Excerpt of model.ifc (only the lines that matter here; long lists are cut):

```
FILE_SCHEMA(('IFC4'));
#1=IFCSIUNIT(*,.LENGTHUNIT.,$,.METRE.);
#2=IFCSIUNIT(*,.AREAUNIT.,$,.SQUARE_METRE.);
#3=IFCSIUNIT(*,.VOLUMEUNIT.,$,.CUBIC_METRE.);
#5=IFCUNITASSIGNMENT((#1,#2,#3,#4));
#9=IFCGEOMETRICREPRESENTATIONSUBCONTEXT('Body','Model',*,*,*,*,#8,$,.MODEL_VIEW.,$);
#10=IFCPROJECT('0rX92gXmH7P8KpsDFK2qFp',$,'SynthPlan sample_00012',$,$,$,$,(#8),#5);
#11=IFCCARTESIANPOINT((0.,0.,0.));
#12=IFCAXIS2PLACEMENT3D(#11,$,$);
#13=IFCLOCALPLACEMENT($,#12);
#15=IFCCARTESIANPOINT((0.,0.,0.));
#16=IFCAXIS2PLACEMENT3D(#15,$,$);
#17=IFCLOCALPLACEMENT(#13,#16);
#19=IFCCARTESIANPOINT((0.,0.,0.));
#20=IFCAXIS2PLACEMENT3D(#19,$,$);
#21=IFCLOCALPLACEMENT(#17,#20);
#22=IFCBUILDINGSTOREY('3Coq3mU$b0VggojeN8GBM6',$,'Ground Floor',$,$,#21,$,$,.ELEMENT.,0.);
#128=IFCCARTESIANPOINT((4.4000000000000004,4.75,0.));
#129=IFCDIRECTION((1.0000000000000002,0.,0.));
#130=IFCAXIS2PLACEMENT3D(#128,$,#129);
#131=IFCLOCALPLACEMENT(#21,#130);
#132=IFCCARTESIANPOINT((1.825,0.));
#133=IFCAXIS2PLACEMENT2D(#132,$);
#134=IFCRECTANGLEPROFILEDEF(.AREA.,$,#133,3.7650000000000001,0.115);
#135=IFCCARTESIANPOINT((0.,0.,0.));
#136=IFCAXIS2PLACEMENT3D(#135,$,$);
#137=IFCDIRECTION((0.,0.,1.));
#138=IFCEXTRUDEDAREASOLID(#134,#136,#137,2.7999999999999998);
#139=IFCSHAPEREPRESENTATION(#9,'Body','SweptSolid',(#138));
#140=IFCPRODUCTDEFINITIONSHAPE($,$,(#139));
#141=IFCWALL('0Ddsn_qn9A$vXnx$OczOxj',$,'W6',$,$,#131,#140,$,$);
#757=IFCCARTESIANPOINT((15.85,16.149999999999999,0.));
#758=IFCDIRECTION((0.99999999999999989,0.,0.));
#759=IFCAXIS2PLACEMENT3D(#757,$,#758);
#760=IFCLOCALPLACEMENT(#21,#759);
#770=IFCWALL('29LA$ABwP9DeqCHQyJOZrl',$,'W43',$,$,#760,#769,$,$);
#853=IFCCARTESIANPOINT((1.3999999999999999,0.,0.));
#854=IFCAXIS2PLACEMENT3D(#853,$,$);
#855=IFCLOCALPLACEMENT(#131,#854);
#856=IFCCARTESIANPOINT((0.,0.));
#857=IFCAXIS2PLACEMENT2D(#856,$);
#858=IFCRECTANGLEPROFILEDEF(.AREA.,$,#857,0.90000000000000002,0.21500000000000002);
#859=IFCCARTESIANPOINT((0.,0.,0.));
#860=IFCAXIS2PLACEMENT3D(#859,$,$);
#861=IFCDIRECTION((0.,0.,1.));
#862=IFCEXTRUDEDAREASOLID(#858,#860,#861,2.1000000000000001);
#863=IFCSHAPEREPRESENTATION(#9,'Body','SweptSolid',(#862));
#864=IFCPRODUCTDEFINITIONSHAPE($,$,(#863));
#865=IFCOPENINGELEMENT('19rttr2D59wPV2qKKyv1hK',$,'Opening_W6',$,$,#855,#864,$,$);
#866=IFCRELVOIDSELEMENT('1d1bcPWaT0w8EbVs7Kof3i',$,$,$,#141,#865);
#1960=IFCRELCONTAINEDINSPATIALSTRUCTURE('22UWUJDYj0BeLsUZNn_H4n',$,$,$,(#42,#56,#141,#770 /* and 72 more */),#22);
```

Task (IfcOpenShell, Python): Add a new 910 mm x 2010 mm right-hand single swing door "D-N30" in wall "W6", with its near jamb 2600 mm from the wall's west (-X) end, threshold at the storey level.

```python
import numpy as np
import ifcopenshell
import ifcopenshell.api.feature
import ifcopenshell.api.geometry
import ifcopenshell.api.root
import ifcopenshell.api.spatial
import ifcopenshell.geom
import ifcopenshell.util.element
import ifcopenshell.util.placement
import ifcopenshell.util.representation
import ifcopenshell.util.shape
import ifcopenshell.util.unit

model = ifcopenshell.open("model.ifc")
unit_scale = ifcopenshell.util.unit.calculate_unit_scale(model)
settings = ifcopenshell.geom.settings()


def volume(element):
    """Net volume in cubic metres, openings subtracted."""
    shape = ifcopenshell.geom.create_shape(settings, element)
    return ifcopenshell.util.shape.get_volume(shape.geometry)


wall = model.by_guid("0Ddsn_qn9A$vXnx$OczOxj")
storey = ifcopenshell.util.element.get_container(wall, ifc_class="IfcBuildingStorey")
context = ifcopenshell.util.representation.get_context(model, "Model", "Body", "MODEL_VIEW")
before = volume(wall)

width, height, from_end, sill = 0.91, 2.01, 2.6, 0.0  # metres

# The wall runs along its own X axis, and the end named is its -X end.
wall_shape = ifcopenshell.geom.create_shape(settings, wall)
x, y, z = ifcopenshell.util.shape.get_vertices(wall_shape.geometry).T
start = x.min() + from_end
face, thickness = float(y.min()), float(y.max() - y.min())
wall_matrix = ifcopenshell.util.placement.get_local_placement(wall.ObjectPlacement)
level = ifcopenshell.util.placement.get_local_placement(storey.ObjectPlacement)[2, 3]


def in_wall(x, y):
    """Placement at x, y metres in the wall's axes, at sill height."""
    matrix = wall_matrix.copy()
    matrix[:, 3] = wall_matrix @ np.array([x / unit_scale, y / unit_scale, 0.0, 1.0])
    matrix[2, 3] = level + sill / unit_scale
    return matrix


# Opening: a box that overshoots both wall faces by 50 mm.
opening = ifcopenshell.api.root.create_entity(model, ifc_class="IfcOpeningElement", predefined_type="OPENING")
box = ifcopenshell.api.geometry.add_wall_representation(
    model, context=context, length=width, height=height, thickness=thickness + 0.1
)
ifcopenshell.api.geometry.assign_representation(model, product=opening, representation=box)
ifcopenshell.api.geometry.edit_object_placement(model, product=opening, matrix=in_wall(start, face - 0.05), is_si=False)
ifcopenshell.api.feature.add_feature(model, feature=opening, element=wall)

door = ifcopenshell.api.root.create_entity(model, ifc_class="IfcDoor", name="D-N30", predefined_type="DOOR")
door.OverallWidth, door.OverallHeight = width / unit_scale, height / unit_scale
door.OperationType = "SINGLE_SWING_RIGHT"
body = ifcopenshell.api.geometry.add_door_representation(
    model,
    context=context,
    overall_width=door.OverallWidth,
    overall_height=door.OverallHeight,
    operation_type="SINGLE_SWING_RIGHT",
    lining_properties={"LiningDepth": thickness / unit_scale, "ThresholdDepth": thickness / unit_scale},
)
ifcopenshell.api.geometry.assign_representation(model, product=door, representation=body)
ifcopenshell.api.spatial.assign_container(model, products=[door], relating_structure=storey)
ifcopenshell.api.feature.add_filling(model, opening=opening, element=door)

# The lining spans the wall, so the door starts at the wall face.
ifcopenshell.api.geometry.edit_object_placement(model, product=door, matrix=in_wall(start, face), is_si=False)

after = volume(wall)

print(f"wall volume {before:.3f} -> {after:.3f} m3")

model.write("model-out.ifc")
```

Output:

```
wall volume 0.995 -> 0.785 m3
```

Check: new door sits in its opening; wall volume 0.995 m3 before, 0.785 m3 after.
